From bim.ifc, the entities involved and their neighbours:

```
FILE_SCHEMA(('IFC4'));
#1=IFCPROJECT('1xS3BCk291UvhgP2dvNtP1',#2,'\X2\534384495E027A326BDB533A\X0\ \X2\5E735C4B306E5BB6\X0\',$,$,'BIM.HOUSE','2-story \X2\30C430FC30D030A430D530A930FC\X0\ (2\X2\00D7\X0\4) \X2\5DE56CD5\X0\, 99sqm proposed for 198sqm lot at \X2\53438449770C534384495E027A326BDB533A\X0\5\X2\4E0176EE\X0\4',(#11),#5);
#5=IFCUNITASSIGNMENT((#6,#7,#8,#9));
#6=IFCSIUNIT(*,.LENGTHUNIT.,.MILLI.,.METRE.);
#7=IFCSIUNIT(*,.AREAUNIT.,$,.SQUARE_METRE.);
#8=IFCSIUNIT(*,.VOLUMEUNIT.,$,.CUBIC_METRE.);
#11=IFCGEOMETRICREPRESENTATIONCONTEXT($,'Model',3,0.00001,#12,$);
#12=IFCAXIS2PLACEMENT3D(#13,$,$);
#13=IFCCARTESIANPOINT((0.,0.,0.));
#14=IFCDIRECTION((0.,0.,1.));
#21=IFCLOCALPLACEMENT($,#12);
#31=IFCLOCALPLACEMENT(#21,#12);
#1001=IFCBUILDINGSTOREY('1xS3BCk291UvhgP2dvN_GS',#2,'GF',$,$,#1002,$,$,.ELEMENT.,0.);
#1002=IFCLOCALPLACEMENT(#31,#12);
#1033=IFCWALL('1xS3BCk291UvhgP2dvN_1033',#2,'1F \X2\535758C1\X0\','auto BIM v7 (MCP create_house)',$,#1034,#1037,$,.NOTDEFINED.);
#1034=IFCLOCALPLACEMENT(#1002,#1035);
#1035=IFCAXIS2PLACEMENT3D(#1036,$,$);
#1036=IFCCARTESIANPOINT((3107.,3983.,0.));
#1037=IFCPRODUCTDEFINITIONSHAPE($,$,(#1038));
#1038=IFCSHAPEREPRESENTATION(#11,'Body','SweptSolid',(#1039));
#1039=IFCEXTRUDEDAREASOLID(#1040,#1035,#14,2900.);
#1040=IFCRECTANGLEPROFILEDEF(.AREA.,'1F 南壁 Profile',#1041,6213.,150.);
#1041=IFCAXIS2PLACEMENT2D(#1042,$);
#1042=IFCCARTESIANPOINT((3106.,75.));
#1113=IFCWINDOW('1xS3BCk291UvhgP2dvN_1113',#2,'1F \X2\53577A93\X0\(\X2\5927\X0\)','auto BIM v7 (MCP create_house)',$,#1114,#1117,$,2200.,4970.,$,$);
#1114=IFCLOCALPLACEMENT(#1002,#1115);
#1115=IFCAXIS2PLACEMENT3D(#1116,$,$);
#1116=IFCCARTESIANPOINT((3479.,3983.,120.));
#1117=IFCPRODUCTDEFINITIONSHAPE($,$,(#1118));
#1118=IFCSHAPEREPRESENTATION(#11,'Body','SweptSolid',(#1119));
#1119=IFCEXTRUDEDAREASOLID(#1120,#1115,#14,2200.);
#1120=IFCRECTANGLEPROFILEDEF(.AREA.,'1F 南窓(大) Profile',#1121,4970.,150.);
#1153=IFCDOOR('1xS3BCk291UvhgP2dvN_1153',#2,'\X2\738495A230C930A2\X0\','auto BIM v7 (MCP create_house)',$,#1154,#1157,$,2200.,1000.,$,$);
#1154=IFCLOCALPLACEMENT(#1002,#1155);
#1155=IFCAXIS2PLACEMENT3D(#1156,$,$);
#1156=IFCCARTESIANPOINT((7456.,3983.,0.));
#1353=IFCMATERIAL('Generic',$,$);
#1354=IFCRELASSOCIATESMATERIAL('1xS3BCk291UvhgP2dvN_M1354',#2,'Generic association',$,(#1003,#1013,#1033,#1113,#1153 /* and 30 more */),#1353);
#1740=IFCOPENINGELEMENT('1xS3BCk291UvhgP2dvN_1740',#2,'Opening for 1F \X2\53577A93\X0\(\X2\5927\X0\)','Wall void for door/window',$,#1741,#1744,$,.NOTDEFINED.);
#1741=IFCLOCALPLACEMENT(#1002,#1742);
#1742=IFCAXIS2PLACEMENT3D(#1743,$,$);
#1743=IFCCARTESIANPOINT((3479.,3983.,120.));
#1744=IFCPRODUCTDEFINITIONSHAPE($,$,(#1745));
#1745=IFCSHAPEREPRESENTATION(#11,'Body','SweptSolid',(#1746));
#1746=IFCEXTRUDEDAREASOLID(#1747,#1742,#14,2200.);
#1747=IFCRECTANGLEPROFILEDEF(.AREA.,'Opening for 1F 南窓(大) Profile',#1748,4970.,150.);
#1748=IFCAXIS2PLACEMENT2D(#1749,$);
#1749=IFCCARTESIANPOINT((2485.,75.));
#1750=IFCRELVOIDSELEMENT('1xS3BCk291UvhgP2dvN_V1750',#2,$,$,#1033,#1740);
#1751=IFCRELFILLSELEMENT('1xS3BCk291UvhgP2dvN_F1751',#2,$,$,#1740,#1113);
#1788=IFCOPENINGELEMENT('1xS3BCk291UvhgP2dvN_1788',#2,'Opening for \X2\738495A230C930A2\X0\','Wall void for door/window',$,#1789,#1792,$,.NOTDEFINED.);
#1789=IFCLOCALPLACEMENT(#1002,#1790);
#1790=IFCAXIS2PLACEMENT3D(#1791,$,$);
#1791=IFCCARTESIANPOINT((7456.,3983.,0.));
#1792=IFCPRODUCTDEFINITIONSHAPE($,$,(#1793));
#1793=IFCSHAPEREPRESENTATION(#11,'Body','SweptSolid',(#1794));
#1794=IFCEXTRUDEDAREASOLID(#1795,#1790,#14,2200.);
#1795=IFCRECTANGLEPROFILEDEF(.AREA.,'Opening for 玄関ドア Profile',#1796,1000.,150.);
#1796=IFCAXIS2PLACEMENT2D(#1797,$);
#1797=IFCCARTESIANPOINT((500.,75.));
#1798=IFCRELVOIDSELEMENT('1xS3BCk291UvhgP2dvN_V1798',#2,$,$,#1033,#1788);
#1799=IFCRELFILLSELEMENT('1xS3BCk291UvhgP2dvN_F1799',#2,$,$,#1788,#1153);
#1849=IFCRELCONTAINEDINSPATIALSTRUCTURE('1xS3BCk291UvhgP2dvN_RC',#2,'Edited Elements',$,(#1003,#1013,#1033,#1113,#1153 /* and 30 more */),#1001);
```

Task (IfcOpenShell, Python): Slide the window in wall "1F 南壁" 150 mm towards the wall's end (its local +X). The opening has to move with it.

```python
import ifcopenshell
import ifcopenshell.api.geometry
import ifcopenshell.util.placement
import ifcopenshell.util.unit

model = ifcopenshell.open("bim.ifc")
unit_scale = ifcopenshell.util.unit.calculate_unit_scale(model)

window = model.by_guid("1xS3BCk291UvhgP2dvN_1113")
opening = window.FillsVoids[0].RelatingOpeningElement
wall = opening.VoidsElements[0].RelatingBuildingElement

wall_matrix = ifcopenshell.util.placement.get_local_placement(wall.ObjectPlacement)
shift = wall_matrix[:3, 0] * 0.15 / unit_scale
before = ifcopenshell.util.placement.get_local_placement(window.ObjectPlacement)[:3, 3].copy()

# The window is not placed relative to its opening, so move both.
for product in (opening, window):
    matrix = ifcopenshell.util.placement.get_local_placement(product.ObjectPlacement)
    matrix[:3, 3] += shift
    ifcopenshell.api.geometry.edit_object_placement(model, product=product, matrix=matrix, is_si=False)

after = ifcopenshell.util.placement.get_local_placement(window.ObjectPlacement)[:3, 3]
print("window moved by", (after - before).round(3) + 0.0)

model.write("bim_rev.ifc")
```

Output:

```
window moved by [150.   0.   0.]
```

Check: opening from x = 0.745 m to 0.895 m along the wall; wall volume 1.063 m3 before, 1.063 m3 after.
